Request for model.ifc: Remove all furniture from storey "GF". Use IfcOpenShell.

First a look at what the model holds.

```python
import ifcopenshell
import ifcopenshell.util.element

model = ifcopenshell.open("model.ifc")
print(model.schema)
storey = next(s for s in model.by_type("IfcBuildingStorey") if s.Name == "GF")
furniture = [e for e in ifcopenshell.util.element.get_decomposition(storey) if e.is_a("IfcFurnishingElement")]
seen = {}
for e in furniture:
    element_type = ifcopenshell.util.element.get_type(e)
    name = element_type.Name if element_type not in (None, e) else None
    seen[name] = seen.get(name, 0) + 1
for name, count in sorted(seen.items(), key=str):
    print(count, "x", name)
```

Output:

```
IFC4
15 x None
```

```python
import ifcopenshell
import ifcopenshell.api.root
import ifcopenshell.util.element

model = ifcopenshell.open("model.ifc")

storey = next(s for s in model.by_type("IfcBuildingStorey") if s.Name == "GF")
furniture = [e for e in ifcopenshell.util.element.get_decomposition(storey) if e.is_a("IfcFurnishingElement")]

for e in furniture:
    ifcopenshell.api.root.remove_product(model, product=e)
print(len(furniture), "removed")

model.write("model_rev.ifc")
```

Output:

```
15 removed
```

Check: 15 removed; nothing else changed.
